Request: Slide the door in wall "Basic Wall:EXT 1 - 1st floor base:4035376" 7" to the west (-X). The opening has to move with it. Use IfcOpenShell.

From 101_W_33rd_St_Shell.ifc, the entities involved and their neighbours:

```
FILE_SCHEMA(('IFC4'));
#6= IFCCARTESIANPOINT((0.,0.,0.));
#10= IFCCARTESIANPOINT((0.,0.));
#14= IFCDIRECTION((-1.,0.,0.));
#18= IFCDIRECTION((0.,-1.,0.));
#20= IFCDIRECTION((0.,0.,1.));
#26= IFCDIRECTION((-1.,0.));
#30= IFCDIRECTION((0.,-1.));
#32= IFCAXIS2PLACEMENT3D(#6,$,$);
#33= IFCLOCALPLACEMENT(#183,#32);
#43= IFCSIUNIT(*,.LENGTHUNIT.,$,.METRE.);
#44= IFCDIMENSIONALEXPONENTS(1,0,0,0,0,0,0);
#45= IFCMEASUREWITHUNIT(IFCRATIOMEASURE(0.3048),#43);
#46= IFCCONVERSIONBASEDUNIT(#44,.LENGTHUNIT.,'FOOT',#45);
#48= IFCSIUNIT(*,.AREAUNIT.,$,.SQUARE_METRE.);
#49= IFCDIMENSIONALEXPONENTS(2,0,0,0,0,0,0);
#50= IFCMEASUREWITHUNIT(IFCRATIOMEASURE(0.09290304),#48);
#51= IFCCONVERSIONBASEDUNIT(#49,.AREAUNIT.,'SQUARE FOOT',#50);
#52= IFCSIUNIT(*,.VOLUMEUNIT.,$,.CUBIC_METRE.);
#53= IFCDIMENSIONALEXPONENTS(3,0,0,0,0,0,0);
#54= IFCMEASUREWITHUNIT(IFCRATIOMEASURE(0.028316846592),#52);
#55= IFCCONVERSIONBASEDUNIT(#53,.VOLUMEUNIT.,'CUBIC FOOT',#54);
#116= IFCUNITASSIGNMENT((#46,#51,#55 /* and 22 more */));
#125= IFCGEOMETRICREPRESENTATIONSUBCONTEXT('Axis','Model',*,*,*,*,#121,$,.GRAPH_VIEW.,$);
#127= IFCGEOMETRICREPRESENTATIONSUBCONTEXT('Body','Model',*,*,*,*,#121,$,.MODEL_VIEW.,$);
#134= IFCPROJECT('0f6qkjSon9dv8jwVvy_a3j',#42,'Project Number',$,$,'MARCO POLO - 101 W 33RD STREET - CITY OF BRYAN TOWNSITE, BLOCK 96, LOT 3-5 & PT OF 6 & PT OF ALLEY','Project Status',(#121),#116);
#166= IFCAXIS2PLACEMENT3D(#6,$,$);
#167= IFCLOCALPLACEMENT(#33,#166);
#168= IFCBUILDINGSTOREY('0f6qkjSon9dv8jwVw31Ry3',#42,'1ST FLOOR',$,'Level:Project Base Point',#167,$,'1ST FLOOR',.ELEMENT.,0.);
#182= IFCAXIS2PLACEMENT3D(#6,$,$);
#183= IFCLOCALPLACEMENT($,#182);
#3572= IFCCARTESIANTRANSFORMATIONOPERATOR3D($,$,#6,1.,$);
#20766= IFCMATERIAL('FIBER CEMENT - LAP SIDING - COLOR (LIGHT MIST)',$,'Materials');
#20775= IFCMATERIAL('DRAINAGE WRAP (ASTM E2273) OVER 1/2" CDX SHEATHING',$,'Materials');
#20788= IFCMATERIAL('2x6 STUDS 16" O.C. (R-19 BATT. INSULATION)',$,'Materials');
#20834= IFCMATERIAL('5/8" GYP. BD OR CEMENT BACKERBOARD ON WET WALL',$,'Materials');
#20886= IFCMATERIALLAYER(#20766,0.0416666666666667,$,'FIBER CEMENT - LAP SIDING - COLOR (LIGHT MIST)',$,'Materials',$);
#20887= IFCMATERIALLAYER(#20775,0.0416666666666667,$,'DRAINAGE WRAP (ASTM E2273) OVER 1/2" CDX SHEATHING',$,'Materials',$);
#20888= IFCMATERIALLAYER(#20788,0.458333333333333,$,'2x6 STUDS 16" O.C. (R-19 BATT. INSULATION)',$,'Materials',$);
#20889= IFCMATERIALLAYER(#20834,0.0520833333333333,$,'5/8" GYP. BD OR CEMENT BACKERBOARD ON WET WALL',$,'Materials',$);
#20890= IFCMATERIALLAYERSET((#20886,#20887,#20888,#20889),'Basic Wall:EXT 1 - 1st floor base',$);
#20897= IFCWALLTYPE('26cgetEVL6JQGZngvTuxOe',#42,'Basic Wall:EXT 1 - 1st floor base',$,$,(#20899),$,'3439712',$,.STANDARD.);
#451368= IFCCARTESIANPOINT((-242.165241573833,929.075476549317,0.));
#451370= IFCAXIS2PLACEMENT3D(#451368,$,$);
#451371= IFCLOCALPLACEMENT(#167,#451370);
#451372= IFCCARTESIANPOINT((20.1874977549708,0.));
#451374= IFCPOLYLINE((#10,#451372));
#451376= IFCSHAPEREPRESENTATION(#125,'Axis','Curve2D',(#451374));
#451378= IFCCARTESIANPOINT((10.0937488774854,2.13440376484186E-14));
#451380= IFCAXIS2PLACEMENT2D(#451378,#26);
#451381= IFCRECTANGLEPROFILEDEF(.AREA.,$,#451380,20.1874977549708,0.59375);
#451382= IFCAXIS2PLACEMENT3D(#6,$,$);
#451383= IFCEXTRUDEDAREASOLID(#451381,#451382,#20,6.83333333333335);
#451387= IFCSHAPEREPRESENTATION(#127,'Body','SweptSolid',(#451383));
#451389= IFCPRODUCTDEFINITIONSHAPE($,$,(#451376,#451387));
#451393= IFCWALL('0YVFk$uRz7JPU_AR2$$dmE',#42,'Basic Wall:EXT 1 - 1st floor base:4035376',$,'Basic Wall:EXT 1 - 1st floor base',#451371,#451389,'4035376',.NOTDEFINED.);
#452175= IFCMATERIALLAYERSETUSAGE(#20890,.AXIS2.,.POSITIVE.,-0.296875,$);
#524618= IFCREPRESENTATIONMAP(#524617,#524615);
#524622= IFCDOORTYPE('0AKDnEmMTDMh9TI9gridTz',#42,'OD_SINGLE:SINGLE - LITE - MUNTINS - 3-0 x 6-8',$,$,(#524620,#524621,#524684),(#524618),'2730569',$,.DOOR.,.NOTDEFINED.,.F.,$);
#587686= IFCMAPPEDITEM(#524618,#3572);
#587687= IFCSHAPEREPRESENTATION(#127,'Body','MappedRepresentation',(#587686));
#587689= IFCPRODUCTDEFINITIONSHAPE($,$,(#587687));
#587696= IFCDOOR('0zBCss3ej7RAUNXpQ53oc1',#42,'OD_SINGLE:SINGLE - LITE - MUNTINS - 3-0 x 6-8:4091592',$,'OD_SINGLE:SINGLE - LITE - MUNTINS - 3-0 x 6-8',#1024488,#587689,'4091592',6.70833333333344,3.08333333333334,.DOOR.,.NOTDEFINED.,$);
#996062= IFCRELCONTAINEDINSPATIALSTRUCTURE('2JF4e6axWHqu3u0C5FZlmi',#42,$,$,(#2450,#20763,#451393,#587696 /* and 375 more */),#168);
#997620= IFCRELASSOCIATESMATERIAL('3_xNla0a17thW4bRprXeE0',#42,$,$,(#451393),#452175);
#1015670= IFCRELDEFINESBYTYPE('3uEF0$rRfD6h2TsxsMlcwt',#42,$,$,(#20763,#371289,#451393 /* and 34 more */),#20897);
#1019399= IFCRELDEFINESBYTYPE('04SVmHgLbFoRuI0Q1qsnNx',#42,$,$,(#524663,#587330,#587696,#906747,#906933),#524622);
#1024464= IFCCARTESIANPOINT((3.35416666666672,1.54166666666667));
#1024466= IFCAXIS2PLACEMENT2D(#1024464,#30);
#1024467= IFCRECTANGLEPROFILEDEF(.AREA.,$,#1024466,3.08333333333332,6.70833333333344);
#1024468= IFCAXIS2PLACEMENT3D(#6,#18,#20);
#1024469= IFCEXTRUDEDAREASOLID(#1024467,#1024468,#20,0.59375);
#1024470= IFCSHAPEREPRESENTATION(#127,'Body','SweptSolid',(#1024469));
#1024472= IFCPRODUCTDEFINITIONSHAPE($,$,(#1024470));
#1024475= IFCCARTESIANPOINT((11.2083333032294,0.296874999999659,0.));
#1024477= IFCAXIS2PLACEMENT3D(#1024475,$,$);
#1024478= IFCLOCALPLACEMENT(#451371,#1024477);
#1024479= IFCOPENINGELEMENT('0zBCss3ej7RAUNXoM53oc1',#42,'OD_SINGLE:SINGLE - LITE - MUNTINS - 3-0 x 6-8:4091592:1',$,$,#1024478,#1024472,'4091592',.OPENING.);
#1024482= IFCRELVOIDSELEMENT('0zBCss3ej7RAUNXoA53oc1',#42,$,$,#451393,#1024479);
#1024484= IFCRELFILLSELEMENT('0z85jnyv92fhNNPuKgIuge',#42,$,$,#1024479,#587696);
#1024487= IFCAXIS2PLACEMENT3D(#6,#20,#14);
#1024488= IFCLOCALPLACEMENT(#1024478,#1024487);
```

```python
import ifcopenshell
import ifcopenshell.api.geometry
import ifcopenshell.util.placement
import ifcopenshell.util.unit

model = ifcopenshell.open("101_W_33rd_St_Shell.ifc")
unit_scale = ifcopenshell.util.unit.calculate_unit_scale(model)

door = model.by_guid("0zBCss3ej7RAUNXpQ53oc1")
opening = door.FillsVoids[0].RelatingOpeningElement
wall = opening.VoidsElements[0].RelatingBuildingElement

wall_matrix = ifcopenshell.util.placement.get_local_placement(wall.ObjectPlacement)
shift = wall_matrix[:3, 0] * -7 * 0.0254 / unit_scale
before = ifcopenshell.util.placement.get_local_placement(door.ObjectPlacement)[:3, 3].copy()

# The door is placed relative to its opening, so it follows when the opening moves.
matrix = ifcopenshell.util.placement.get_local_placement(opening.ObjectPlacement)
matrix[:3, 3] += shift
ifcopenshell.api.geometry.edit_object_placement(
    model, product=opening, matrix=matrix, is_si=False, should_transform_children=True
)

after = ifcopenshell.util.placement.get_local_placement(door.ObjectPlacement)[:3, 3]
print("door moved by", (after - before).round(3) + 0.0)

model.write("101_W_33rd_St_Shell_updated.ifc")
```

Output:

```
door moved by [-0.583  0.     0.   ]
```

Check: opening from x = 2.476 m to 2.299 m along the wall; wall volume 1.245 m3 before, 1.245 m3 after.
